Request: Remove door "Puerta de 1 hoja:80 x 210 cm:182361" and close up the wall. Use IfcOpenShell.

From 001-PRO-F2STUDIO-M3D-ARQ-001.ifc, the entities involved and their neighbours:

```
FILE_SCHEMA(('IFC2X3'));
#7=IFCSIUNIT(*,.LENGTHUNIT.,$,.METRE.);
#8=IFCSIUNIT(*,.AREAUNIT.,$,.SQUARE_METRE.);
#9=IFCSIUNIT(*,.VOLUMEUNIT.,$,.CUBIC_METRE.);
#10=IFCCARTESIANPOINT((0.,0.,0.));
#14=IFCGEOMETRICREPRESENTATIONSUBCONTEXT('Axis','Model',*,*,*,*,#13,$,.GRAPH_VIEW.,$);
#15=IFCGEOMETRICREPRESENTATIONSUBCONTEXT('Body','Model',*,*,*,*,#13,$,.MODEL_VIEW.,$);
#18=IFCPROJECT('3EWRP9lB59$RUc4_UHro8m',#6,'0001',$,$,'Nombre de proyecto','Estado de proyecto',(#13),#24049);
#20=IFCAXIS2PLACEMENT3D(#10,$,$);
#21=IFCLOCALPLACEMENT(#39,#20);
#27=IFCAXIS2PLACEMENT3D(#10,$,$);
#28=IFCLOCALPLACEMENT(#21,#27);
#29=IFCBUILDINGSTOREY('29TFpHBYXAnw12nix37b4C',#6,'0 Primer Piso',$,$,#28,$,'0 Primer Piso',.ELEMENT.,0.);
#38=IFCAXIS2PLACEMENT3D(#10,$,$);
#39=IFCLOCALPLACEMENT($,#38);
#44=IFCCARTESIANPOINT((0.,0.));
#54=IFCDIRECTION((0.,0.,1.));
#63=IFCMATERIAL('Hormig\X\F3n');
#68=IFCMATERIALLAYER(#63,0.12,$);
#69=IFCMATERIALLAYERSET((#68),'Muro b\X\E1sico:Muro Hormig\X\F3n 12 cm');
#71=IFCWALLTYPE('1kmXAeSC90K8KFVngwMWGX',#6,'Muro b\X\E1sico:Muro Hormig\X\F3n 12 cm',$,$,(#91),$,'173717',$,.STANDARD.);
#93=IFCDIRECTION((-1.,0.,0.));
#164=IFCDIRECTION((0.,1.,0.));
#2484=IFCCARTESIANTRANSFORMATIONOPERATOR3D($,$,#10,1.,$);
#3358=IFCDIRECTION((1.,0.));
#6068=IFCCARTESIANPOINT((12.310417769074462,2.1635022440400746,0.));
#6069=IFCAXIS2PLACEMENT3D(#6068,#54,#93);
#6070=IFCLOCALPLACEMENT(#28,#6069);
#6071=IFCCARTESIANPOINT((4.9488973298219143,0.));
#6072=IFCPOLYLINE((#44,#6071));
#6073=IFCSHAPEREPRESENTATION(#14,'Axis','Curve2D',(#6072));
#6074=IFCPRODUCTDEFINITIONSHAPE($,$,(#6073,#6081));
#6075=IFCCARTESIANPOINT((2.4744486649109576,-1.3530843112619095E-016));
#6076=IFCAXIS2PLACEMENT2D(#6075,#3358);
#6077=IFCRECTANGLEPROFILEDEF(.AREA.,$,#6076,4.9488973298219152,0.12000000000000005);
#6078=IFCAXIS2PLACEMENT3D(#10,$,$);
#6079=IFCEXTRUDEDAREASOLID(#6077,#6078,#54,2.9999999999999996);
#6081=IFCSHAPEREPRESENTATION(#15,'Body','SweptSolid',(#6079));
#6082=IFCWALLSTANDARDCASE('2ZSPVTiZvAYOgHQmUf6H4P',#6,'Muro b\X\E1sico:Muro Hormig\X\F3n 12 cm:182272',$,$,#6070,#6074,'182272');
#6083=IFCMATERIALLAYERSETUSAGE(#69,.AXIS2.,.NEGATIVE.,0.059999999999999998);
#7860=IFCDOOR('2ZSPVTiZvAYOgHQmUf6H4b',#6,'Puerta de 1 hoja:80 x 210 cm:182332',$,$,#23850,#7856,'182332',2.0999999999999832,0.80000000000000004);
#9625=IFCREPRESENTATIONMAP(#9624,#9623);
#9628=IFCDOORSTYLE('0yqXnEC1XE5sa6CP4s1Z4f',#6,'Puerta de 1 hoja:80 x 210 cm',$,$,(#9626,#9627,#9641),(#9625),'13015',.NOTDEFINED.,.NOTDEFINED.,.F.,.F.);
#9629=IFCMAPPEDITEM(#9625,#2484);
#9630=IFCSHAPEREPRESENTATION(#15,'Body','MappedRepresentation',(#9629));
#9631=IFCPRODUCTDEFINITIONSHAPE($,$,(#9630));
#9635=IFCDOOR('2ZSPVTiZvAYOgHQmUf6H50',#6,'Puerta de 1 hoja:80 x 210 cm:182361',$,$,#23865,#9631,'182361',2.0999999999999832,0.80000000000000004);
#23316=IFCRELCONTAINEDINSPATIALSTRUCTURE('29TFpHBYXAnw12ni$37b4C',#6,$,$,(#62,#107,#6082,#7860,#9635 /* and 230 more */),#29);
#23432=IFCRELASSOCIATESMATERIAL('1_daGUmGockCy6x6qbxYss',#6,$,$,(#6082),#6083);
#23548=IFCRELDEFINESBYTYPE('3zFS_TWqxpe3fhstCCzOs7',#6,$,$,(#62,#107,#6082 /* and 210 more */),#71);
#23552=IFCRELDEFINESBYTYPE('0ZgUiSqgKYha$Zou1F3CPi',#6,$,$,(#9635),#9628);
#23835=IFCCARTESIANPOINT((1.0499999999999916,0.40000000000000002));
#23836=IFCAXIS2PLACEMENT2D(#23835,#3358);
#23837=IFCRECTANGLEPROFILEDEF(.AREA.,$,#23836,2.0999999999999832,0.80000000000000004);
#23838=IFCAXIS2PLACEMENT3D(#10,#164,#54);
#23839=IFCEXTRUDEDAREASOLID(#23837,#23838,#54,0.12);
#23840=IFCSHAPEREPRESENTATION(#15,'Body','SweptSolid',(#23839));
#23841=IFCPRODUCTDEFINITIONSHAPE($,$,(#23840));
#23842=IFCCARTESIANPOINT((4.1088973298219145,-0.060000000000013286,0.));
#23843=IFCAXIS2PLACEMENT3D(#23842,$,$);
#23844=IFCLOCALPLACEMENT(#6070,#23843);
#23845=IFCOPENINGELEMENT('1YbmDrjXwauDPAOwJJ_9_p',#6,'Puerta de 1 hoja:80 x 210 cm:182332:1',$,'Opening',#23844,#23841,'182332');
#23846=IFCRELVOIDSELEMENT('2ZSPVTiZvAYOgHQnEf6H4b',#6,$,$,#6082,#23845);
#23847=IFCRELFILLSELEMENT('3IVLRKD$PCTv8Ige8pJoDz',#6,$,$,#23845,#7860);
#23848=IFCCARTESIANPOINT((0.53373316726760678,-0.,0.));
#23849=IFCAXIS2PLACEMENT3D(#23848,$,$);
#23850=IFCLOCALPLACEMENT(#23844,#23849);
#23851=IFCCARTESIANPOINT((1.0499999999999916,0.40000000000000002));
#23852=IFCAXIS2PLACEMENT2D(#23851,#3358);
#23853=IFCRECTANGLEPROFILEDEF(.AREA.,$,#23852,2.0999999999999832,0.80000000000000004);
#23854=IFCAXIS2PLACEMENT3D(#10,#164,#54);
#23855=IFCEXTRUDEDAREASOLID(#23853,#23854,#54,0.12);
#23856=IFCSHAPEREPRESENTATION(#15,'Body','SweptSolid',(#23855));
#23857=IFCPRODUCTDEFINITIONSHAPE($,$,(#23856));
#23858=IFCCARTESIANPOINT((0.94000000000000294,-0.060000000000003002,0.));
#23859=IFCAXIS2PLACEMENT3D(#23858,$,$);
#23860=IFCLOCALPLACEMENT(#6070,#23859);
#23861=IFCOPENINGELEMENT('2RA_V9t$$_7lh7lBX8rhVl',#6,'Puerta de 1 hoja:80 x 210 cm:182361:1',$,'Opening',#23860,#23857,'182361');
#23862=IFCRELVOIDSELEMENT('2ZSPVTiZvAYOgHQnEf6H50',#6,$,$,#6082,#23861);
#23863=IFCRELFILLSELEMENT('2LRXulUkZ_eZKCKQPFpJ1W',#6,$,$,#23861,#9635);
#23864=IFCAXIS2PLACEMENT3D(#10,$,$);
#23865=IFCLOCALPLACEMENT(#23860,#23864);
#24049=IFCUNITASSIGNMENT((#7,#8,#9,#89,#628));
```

```python
import ifcopenshell
import ifcopenshell.api.feature
import ifcopenshell.api.root
import ifcopenshell.geom
import ifcopenshell.util.shape

model = ifcopenshell.open("001-PRO-F2STUDIO-M3D-ARQ-001.ifc")
settings = ifcopenshell.geom.settings()


def volume(element):
    """Net volume in cubic metres, openings subtracted."""
    shape = ifcopenshell.geom.create_shape(settings, element)
    return ifcopenshell.util.shape.get_volume(shape.geometry)


door = model.by_guid("2ZSPVTiZvAYOgHQmUf6H50")
opening = door.FillsVoids[0].RelatingOpeningElement
wall = opening.VoidsElements[0].RelatingBuildingElement
before = volume(wall)

ifcopenshell.api.root.remove_product(model, product=door)
ifcopenshell.api.feature.remove_feature(model, feature=opening)

after = volume(wall)

print(f"wall volume {before:.3f} -> {after:.3f} m3")

model.write("001-PRO-F2STUDIO-M3D-ARQ-001-out.ifc")
```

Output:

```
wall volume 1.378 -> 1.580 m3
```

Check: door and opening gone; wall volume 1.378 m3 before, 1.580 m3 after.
